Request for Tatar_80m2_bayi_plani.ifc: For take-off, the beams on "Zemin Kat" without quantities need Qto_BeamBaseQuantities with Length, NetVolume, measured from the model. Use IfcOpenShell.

First a look at what the model holds.

```python
import ifcopenshell
import ifcopenshell.util.element
import ifcopenshell.util.unit

model = ifcopenshell.open("Tatar_80m2_bayi_plani.ifc")
print(model.schema)
for unit_type in ("LENGTHUNIT", "AREAUNIT", "VOLUMEUNIT"):
    print(unit_type, ifcopenshell.util.unit.calculate_unit_scale(model, unit_type))
storey = next(s for s in model.by_type("IfcBuildingStorey") if s.Name == "Zemin Kat")
beams = [e for e in ifcopenshell.util.element.get_decomposition(storey) if e.is_a("IfcBeam")]
for e in sorted(beams, key=lambda e: e.id()):
    print(e.id(), e.is_a(), e.Name, list(ifcopenshell.util.element.get_psets(e, qtos_only=True)), sep=" | ")
```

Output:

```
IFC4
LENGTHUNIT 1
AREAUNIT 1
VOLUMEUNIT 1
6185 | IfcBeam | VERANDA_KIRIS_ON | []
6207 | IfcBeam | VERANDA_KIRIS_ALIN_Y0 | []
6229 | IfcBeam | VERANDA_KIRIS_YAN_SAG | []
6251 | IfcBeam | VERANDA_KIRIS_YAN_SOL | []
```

```python
import ifcopenshell
import ifcopenshell.api.pset
import ifcopenshell.geom
import ifcopenshell.util.element
import ifcopenshell.util.shape
import ifcopenshell.util.unit

model = ifcopenshell.open("Tatar_80m2_bayi_plani.ifc")
unit_scale = ifcopenshell.util.unit.calculate_unit_scale(model)
volume_scale = ifcopenshell.util.unit.calculate_unit_scale(model, "VOLUMEUNIT")
settings = ifcopenshell.geom.settings()

storey = next(s for s in model.by_type("IfcBuildingStorey") if s.Name == "Zemin Kat")
beams = [e for e in ifcopenshell.util.element.get_decomposition(storey) if e.is_a("IfcBeam")]

for e in sorted(beams, key=lambda e: e.id()):
    if ifcopenshell.util.element.get_psets(e, qtos_only=True, should_inherit=False):
        continue
    # Geometry comes back in metres, in the element's own axes.
    shape = ifcopenshell.geom.create_shape(settings, e)
    values = {
        "Length": ifcopenshell.util.shape.get_max_xyz(shape.geometry) / unit_scale,
        "NetVolume": ifcopenshell.util.shape.get_volume(shape.geometry) / volume_scale,
    }
    qto = ifcopenshell.api.pset.add_qto(model, product=e, name="Qto_BeamBaseQuantities")
    ifcopenshell.api.pset.edit_qto(model, qto=qto, properties=values)
    print(e.id(), {k: round(v, 3) for k, v in values.items()})

model.write("Tatar_80m2_bayi_plani_updated.ifc")
```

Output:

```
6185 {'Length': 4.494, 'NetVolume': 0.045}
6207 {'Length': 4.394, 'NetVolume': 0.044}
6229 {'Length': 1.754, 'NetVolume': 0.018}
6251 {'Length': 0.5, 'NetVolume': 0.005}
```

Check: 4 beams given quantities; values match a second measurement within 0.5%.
